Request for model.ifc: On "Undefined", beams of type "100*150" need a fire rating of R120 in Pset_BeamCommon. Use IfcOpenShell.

First a look at what the model holds.

```python
import ifcopenshell
import ifcopenshell.util.element

model = ifcopenshell.open("model.ifc")
print(model.schema)
storey = next(s for s in model.by_type("IfcBuildingStorey") if s.Name == "Undefined")
beams = [e for e in ifcopenshell.util.element.get_decomposition(storey) if e.is_a("IfcBeam")]
seen = {}
for e in beams:
    element_type = ifcopenshell.util.element.get_type(e)
    key = (element_type.Name if element_type != e and element_type else None, ifcopenshell.util.element.get_pset(e, "Pset_BeamCommon", "FireRating"))
    seen[key] = seen.get(key, 0) + 1
for (name, value), count in sorted(seen.items(), key=str):
    print(count, "x", name, "|", value)
```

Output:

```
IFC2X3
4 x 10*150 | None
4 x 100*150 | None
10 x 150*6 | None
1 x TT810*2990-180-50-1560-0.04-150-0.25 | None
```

```python
import ifcopenshell
import ifcopenshell.api.pset
import ifcopenshell.util.element

model = ifcopenshell.open("model.ifc")

storey = next(s for s in model.by_type("IfcBuildingStorey") if s.Name == "Undefined")
beams = [e for e in ifcopenshell.util.element.get_decomposition(storey) if e.is_a("IfcBeam")]

count = 0
for e in beams:
    element_type = ifcopenshell.util.element.get_type(e)
    if element_type in (None, e) or element_type.Name != "100*150":
        continue
    # add_pset returns the element's existing set when there is one.
    pset = ifcopenshell.api.pset.add_pset(model, product=e, name="Pset_BeamCommon")
    ifcopenshell.api.pset.edit_pset(model, pset=pset, properties={"FireRating": "R120"})
    count += 1

print(count, "beams updated")

model.write("model_v2.ifc")
```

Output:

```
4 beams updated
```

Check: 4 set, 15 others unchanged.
